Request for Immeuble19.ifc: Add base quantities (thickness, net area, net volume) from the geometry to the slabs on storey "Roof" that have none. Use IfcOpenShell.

First a look at what the model holds.

```python
import ifcopenshell
import ifcopenshell.util.element
import ifcopenshell.util.unit

model = ifcopenshell.open("Immeuble19.ifc")
print(model.schema)
for unit_type in ("LENGTHUNIT", "AREAUNIT", "VOLUMEUNIT"):
    print(unit_type, ifcopenshell.util.unit.calculate_unit_scale(model, unit_type))
storey = next(s for s in model.by_type("IfcBuildingStorey") if s.Name == "Roof")
slabs = [e for e in ifcopenshell.util.element.get_decomposition(storey) if e.is_a("IfcSlab")]
for e in sorted(slabs, key=lambda e: e.id()):
    print(e.id(), e.is_a(), e.Name, list(ifcopenshell.util.element.get_psets(e, qtos_only=True)), sep=" | ")
```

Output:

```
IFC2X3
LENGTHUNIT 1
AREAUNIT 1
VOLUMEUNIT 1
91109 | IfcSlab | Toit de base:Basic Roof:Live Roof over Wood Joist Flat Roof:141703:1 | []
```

```python
import ifcopenshell
import ifcopenshell.api.pset
import ifcopenshell.geom
import ifcopenshell.util.element
import ifcopenshell.util.shape
import ifcopenshell.util.unit

model = ifcopenshell.open("Immeuble19.ifc")
unit_scale = ifcopenshell.util.unit.calculate_unit_scale(model)
area_scale = ifcopenshell.util.unit.calculate_unit_scale(model, "AREAUNIT")
volume_scale = ifcopenshell.util.unit.calculate_unit_scale(model, "VOLUMEUNIT")
settings = ifcopenshell.geom.settings()

storey = next(s for s in model.by_type("IfcBuildingStorey") if s.Name == "Roof")
slabs = [e for e in ifcopenshell.util.element.get_decomposition(storey) if e.is_a("IfcSlab")]

for e in sorted(slabs, key=lambda e: e.id()):
    if ifcopenshell.util.element.get_psets(e, qtos_only=True, should_inherit=False):
        continue
    # Geometry comes back in metres, in the element's own axes.
    shape = ifcopenshell.geom.create_shape(settings, e)
    values = {
        "Width": ifcopenshell.util.shape.get_z(shape.geometry) / unit_scale,
        "NetArea": ifcopenshell.util.shape.get_footprint_area(shape.geometry) / area_scale,
        "NetVolume": ifcopenshell.util.shape.get_volume(shape.geometry) / volume_scale,
    }
    qto = ifcopenshell.api.pset.add_qto(model, product=e, name="BaseQuantities")
    ifcopenshell.api.pset.edit_qto(model, qto=qto, properties=values)
    print(e.id(), {k: round(v, 3) for k, v in values.items()})

model.write("Immeuble19-out.ifc")
```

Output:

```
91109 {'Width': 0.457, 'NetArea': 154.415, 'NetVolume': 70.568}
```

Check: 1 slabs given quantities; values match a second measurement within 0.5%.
